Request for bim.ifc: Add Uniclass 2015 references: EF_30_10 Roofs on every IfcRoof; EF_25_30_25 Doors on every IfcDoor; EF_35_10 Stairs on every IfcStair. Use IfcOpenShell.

First a look at what the model holds.

```python
import ifcopenshell

model = ifcopenshell.open("bim.ifc")
print(model.schema)
print("classifications:", [c.Name for c in model.by_type("IfcClassification")])
for ifc_class in ("IfcDoor", "IfcRoof", "IfcStair", "IfcWall", "IfcWindow"):
    print(ifc_class, len(model.by_type(ifc_class)))
```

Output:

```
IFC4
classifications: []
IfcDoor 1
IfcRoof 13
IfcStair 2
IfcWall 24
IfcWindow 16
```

```python
import ifcopenshell
import ifcopenshell.api.classification

model = ifcopenshell.open("bim.ifc")

system = ifcopenshell.api.classification.add_classification(model, classification="Uniclass 2015")

codes = {
    "IfcRoof": ("EF_30_10", "Roofs"),
    "IfcDoor": ("EF_25_30_25", "Doors"),
    "IfcStair": ("EF_35_10", "Stairs"),
}
for ifc_class, (code, name) in codes.items():
    products = model.by_type(ifc_class)
    ifcopenshell.api.classification.add_reference(
        model, products=products, classification=system, identification=code, name=name
    )
    print(code, len(products))

model.write("bim_edited.ifc")
```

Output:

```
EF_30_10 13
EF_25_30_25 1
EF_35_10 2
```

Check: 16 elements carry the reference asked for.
